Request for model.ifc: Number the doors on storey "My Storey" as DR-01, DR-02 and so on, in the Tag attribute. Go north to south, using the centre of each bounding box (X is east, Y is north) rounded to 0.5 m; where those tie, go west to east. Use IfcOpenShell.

First a look at what the model holds.

```python
import ifcopenshell
import ifcopenshell.util.element
import ifcopenshell.util.placement

model = ifcopenshell.open("model.ifc")
print(model.schema)
storey = next(s for s in model.by_type("IfcBuildingStorey") if s.Name == "My Storey")
doors = [e for e in ifcopenshell.util.element.get_decomposition(storey) if e.is_a("IfcDoor")]
for e in sorted(doors, key=lambda e: e.id()):
    origin = ifcopenshell.util.placement.get_local_placement(e.ObjectPlacement)[:3, 3]
    print(e.id(), e.Tag, e.Name, origin.round(2) + 0.0, sep=" | ")
```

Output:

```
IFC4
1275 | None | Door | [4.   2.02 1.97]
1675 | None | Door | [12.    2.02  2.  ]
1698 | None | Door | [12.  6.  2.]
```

```python
import ifcopenshell
import ifcopenshell.geom
import ifcopenshell.util.element
import ifcopenshell.util.shape

model = ifcopenshell.open("model.ifc")
settings = ifcopenshell.geom.settings()
settings.set("use-world-coords", True)


def centre(element):
    shape = ifcopenshell.geom.create_shape(settings, element)
    return ifcopenshell.util.shape.get_bbox_centroid(shape.geometry)


storey = next(s for s in model.by_type("IfcBuildingStorey") if s.Name == "My Storey")
doors = [e for e in ifcopenshell.util.element.get_decomposition(storey) if e.is_a("IfcDoor")]

# Insertion points can sit at a corner or the storey origin, so sort by the geometry (in metres).
centres = {e: centre(e) for e in doors}
doors.sort(key=lambda e: (-round(centres[e][1] / 0.5), centres[e][0]))

for i, e in enumerate(doors, start=1):
    number = f"DR-{i:02d}"
    e.Tag = number
    print(e.id(), number)

model.write("model_edited.ifc")
```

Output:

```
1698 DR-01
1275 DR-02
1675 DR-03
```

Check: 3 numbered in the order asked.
